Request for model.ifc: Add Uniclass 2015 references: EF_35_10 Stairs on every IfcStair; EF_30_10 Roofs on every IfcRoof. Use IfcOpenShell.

First a look at what the model holds.

```python
import ifcopenshell

model = ifcopenshell.open("model.ifc")
print(model.schema)
print("classifications:", [c.Name for c in model.by_type("IfcClassification")])
for ifc_class in ("IfcDoor", "IfcRoof", "IfcStair", "IfcWall", "IfcWindow"):
    print(ifc_class, len(model.by_type(ifc_class)))
```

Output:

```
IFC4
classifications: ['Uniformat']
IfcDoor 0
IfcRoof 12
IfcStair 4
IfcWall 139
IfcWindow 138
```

```python
import ifcopenshell
import ifcopenshell.api.classification

model = ifcopenshell.open("model.ifc")

system = ifcopenshell.api.classification.add_classification(model, classification="Uniclass 2015")

codes = {
    "IfcStair": ("EF_35_10", "Stairs"),
    "IfcRoof": ("EF_30_10", "Roofs"),
}
for ifc_class, (code, name) in codes.items():
    products = model.by_type(ifc_class)
    ifcopenshell.api.classification.add_reference(
        model, products=products, classification=system, identification=code, name=name
    )
    print(code, len(products))

model.write("model_edited.ifc")
```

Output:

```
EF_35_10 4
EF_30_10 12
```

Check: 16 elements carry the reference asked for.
